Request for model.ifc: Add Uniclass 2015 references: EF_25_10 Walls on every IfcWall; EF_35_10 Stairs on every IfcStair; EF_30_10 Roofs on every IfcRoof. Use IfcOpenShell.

First a look at what the model holds.

```python
import ifcopenshell

model = ifcopenshell.open("model.ifc")
print(model.schema)
print("classifications:", [c.Name for c in model.by_type("IfcClassification")])
for ifc_class in ("IfcDoor", "IfcRoof", "IfcStair", "IfcWall", "IfcWindow"):
    print(ifc_class, len(model.by_type(ifc_class)))
```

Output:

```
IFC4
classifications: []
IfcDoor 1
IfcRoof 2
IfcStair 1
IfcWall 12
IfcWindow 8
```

```python
import ifcopenshell
import ifcopenshell.api.classification

model = ifcopenshell.open("model.ifc")

system = ifcopenshell.api.classification.add_classification(model, classification="Uniclass 2015")

codes = {
    "IfcWall": ("EF_25_10", "Walls"),
    "IfcStair": ("EF_35_10", "Stairs"),
    "IfcRoof": ("EF_30_10", "Roofs"),
}
for ifc_class, (code, name) in codes.items():
    products = model.by_type(ifc_class)
    ifcopenshell.api.classification.add_reference(
        model, products=products, classification=system, identification=code, name=name
    )
    print(code, len(products))

model.write("model_edited.ifc")
```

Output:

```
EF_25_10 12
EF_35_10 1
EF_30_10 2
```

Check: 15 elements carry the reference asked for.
